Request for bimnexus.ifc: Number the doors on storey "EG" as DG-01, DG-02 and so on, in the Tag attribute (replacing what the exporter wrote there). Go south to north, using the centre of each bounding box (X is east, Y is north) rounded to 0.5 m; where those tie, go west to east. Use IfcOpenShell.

First a look at what the model holds.

```python
import ifcopenshell
import ifcopenshell.util.element
import ifcopenshell.util.placement

model = ifcopenshell.open("bimnexus.ifc")
print(model.schema)
storey = next(s for s in model.by_type("IfcBuildingStorey") if s.Name == "EG")
doors = [e for e in ifcopenshell.util.element.get_decomposition(storey) if e.is_a("IfcDoor")]
for e in sorted(doors, key=lambda e: e.id()):
    origin = ifcopenshell.util.placement.get_local_placement(e.ObjectPlacement)[:3, 3]
    print(e.id(), e.Tag, e.Name, origin.round(2) + 0.0, sep=" | ")
```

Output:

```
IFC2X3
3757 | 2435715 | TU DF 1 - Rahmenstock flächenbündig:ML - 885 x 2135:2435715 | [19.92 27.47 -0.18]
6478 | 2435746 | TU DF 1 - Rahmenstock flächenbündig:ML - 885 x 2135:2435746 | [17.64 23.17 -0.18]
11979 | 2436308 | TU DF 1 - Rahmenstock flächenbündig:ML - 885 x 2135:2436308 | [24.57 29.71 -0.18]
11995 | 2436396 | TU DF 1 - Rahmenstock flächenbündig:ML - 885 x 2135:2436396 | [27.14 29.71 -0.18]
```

```python
import ifcopenshell
import ifcopenshell.geom
import ifcopenshell.util.element
import ifcopenshell.util.shape

model = ifcopenshell.open("bimnexus.ifc")
settings = ifcopenshell.geom.settings()
settings.set("use-world-coords", True)


def centre(element):
    shape = ifcopenshell.geom.create_shape(settings, element)
    return ifcopenshell.util.shape.get_bbox_centroid(shape.geometry)


storey = next(s for s in model.by_type("IfcBuildingStorey") if s.Name == "EG")
doors = [e for e in ifcopenshell.util.element.get_decomposition(storey) if e.is_a("IfcDoor")]

# Insertion points can sit at a corner or the storey origin, so sort by the geometry (in metres).
centres = {e: centre(e) for e in doors}
doors.sort(key=lambda e: (round(centres[e][1] / 0.5), centres[e][0]))

for i, e in enumerate(doors, start=1):
    number = f"DG-{i:02d}"
    e.Tag = number
    print(e.id(), number)

model.write("bimnexus_updated.ifc")
```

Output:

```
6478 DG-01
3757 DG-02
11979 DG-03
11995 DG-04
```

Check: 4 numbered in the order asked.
